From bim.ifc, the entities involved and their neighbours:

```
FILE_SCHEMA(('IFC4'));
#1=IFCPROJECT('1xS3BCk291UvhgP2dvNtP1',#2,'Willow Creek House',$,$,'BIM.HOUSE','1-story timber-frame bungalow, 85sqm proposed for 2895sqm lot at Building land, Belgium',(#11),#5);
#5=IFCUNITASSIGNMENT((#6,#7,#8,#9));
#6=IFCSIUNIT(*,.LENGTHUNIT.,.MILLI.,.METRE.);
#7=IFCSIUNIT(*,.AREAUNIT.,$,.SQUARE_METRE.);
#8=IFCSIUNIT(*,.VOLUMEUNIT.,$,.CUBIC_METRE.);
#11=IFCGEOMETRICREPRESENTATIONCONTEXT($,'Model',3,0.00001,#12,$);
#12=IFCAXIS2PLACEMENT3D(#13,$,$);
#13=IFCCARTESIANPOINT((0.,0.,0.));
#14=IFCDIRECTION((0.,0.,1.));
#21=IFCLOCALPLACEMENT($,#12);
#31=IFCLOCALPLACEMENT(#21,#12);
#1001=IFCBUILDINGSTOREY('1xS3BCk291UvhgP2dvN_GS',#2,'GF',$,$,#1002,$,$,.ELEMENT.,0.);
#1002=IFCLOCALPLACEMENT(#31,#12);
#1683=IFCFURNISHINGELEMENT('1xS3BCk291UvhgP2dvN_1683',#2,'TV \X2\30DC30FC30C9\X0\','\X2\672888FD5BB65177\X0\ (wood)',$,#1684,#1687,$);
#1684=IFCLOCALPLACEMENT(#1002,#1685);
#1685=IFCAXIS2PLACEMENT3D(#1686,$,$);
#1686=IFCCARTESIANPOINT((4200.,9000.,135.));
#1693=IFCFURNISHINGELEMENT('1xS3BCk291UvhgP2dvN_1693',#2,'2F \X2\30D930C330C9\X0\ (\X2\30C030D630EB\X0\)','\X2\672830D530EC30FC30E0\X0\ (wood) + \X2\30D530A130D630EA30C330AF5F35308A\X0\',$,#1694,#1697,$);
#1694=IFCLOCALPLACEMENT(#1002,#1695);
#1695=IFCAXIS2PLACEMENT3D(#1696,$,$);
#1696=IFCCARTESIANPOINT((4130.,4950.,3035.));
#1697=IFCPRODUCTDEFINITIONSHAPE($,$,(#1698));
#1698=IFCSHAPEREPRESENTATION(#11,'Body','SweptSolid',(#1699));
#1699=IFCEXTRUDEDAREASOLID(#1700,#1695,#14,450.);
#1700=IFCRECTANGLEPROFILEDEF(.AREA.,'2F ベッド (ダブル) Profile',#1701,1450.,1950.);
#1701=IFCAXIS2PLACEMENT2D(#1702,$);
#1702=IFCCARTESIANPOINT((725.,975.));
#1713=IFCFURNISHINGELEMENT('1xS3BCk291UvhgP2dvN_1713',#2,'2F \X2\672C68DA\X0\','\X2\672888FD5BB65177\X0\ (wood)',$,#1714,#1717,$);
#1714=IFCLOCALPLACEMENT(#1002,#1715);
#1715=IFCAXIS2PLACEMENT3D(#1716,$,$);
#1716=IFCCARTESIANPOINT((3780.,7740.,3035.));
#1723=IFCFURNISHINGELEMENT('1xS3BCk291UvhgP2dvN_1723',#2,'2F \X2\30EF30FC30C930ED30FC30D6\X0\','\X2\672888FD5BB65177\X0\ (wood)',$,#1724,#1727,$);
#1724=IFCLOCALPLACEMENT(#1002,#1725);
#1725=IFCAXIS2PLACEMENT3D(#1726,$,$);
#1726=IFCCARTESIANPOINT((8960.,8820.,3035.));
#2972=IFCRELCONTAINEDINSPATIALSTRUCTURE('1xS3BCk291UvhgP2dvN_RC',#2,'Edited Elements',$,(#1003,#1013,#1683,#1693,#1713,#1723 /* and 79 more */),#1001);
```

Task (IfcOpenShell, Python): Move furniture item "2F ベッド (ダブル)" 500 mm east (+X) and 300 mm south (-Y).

```python
import ifcopenshell
import ifcopenshell.api.geometry
import ifcopenshell.util.placement
import ifcopenshell.util.unit

model = ifcopenshell.open("bim.ifc")
unit_scale = ifcopenshell.util.unit.calculate_unit_scale(model)

item = model.by_id(1693)
matrix = ifcopenshell.util.placement.get_local_placement(item.ObjectPlacement)
matrix[0, 3] += 0.5 / unit_scale
matrix[1, 3] -= 0.3 / unit_scale
ifcopenshell.api.geometry.edit_object_placement(model, product=item, matrix=matrix, is_si=False)

print(ifcopenshell.util.placement.get_local_placement(item.ObjectPlacement).round(3) + 0.0)

model.write("bim-out.ifc")
```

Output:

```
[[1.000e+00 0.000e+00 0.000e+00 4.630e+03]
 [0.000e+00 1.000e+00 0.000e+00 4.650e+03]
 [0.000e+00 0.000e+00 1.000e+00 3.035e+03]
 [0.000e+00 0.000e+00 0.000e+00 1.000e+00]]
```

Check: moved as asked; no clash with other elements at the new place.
